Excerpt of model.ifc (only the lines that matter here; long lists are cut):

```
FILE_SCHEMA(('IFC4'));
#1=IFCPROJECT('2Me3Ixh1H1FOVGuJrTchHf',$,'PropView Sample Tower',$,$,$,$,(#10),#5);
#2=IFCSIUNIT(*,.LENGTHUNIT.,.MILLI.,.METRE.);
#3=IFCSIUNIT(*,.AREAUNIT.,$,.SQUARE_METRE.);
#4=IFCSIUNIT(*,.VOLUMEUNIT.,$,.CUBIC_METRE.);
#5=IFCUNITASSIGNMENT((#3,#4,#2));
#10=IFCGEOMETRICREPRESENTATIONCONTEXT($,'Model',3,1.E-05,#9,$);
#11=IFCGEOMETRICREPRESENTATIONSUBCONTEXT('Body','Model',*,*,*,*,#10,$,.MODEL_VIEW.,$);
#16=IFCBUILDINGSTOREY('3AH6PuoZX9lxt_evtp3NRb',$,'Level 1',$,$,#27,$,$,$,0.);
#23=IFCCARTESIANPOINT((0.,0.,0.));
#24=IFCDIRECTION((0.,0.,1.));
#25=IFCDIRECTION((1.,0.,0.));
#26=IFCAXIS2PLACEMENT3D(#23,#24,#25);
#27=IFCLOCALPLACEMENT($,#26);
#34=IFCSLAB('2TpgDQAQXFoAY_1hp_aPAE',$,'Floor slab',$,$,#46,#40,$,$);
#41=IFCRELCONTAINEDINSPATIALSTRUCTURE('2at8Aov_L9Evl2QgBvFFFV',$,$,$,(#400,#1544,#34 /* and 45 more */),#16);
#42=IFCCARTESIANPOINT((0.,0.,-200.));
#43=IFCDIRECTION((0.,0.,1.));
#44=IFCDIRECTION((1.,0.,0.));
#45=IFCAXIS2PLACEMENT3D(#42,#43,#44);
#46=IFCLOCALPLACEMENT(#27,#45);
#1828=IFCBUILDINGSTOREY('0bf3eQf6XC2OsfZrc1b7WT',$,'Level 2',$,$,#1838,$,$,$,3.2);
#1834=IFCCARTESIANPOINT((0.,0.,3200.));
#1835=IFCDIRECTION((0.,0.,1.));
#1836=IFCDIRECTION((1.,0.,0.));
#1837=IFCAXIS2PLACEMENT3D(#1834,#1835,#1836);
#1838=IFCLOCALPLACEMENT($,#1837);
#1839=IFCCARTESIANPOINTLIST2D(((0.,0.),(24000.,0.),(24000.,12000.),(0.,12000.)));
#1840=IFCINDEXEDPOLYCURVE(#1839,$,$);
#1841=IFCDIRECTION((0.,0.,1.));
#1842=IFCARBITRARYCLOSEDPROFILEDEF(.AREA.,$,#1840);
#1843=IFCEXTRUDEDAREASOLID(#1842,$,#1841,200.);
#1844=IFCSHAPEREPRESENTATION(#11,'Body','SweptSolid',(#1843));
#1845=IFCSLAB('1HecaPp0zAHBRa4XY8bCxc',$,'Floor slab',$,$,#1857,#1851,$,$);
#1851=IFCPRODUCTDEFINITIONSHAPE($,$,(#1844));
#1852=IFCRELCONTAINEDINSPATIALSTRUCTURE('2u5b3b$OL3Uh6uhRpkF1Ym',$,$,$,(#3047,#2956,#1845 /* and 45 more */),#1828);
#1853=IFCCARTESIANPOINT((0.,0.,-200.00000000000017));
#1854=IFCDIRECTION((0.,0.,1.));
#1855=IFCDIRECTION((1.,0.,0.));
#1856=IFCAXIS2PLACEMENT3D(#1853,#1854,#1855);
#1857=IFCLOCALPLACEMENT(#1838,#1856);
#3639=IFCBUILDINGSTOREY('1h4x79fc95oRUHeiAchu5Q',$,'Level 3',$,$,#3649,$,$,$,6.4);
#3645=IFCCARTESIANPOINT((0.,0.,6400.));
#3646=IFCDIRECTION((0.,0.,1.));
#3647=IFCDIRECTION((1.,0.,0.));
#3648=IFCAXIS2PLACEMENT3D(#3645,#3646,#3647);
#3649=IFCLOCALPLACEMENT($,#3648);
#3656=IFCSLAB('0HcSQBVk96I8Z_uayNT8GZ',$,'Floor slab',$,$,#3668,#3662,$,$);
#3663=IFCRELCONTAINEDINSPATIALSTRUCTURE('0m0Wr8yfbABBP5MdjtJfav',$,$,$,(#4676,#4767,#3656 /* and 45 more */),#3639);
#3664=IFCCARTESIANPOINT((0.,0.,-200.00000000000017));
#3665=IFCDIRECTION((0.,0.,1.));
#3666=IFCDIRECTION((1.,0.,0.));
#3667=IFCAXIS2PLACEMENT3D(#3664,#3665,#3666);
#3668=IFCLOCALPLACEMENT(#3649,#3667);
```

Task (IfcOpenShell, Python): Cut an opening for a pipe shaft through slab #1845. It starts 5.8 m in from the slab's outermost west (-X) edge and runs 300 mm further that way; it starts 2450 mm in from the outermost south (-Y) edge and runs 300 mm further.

```python
import numpy as np
import ifcopenshell
import ifcopenshell.api.feature
import ifcopenshell.api.geometry
import ifcopenshell.api.root
import ifcopenshell.geom
import ifcopenshell.util.placement
import ifcopenshell.util.representation
import ifcopenshell.util.shape
import ifcopenshell.util.unit

model = ifcopenshell.open("model.ifc")
unit_scale = ifcopenshell.util.unit.calculate_unit_scale(model)
settings = ifcopenshell.geom.settings()


def volume(element):
    """Net volume in cubic metres, openings subtracted."""
    shape = ifcopenshell.geom.create_shape(settings, element)
    return ifcopenshell.util.shape.get_volume(shape.geometry)


slab = model.by_guid("1HecaPp0zAHBRa4XY8bCxc")
before = volume(slab)

# Extent in the slab's own axes, in metres. The edges named are its -X and -Y sides.
slab_shape = ifcopenshell.geom.create_shape(settings, slab)
vertices = ifcopenshell.util.shape.get_vertices(slab_shape.geometry)
x_min, y_min, bottom = vertices.min(axis=0)
top = vertices[:, 2].max()

opening = ifcopenshell.api.root.create_entity(model, ifc_class="IfcOpeningElement", name="Pipe shaft opening", predefined_type="OPENING")
context = ifcopenshell.util.representation.get_context(model, "Model", "Body", "MODEL_VIEW")
width, depth = 0.3, 0.3
outline = [(0.0, 0.0), (width, 0.0), (width, depth), (0.0, depth), (0.0, 0.0)]
# Overshoot both faces by 50 mm so the cut is clean.
shape = ifcopenshell.api.geometry.add_slab_representation(
    model, context=context, depth=top - bottom + 0.1, polyline=outline
)
ifcopenshell.api.geometry.assign_representation(model, product=opening, representation=shape)

matrix = ifcopenshell.util.placement.get_local_placement(slab.ObjectPlacement)
matrix[:, 3] = matrix @ np.append(np.array([x_min + 5.8, y_min + 2.45, bottom - 0.05]) / unit_scale, 1.0)
ifcopenshell.api.geometry.edit_object_placement(model, product=opening, matrix=matrix, is_si=False)
ifcopenshell.api.feature.add_feature(model, feature=opening, element=slab)

after = volume(slab)

print(f"slab volume {before:.3f} -> {after:.3f} m3")

model.write("model_updated.ifc")
```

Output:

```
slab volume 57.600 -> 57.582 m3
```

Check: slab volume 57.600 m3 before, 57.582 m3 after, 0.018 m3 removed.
